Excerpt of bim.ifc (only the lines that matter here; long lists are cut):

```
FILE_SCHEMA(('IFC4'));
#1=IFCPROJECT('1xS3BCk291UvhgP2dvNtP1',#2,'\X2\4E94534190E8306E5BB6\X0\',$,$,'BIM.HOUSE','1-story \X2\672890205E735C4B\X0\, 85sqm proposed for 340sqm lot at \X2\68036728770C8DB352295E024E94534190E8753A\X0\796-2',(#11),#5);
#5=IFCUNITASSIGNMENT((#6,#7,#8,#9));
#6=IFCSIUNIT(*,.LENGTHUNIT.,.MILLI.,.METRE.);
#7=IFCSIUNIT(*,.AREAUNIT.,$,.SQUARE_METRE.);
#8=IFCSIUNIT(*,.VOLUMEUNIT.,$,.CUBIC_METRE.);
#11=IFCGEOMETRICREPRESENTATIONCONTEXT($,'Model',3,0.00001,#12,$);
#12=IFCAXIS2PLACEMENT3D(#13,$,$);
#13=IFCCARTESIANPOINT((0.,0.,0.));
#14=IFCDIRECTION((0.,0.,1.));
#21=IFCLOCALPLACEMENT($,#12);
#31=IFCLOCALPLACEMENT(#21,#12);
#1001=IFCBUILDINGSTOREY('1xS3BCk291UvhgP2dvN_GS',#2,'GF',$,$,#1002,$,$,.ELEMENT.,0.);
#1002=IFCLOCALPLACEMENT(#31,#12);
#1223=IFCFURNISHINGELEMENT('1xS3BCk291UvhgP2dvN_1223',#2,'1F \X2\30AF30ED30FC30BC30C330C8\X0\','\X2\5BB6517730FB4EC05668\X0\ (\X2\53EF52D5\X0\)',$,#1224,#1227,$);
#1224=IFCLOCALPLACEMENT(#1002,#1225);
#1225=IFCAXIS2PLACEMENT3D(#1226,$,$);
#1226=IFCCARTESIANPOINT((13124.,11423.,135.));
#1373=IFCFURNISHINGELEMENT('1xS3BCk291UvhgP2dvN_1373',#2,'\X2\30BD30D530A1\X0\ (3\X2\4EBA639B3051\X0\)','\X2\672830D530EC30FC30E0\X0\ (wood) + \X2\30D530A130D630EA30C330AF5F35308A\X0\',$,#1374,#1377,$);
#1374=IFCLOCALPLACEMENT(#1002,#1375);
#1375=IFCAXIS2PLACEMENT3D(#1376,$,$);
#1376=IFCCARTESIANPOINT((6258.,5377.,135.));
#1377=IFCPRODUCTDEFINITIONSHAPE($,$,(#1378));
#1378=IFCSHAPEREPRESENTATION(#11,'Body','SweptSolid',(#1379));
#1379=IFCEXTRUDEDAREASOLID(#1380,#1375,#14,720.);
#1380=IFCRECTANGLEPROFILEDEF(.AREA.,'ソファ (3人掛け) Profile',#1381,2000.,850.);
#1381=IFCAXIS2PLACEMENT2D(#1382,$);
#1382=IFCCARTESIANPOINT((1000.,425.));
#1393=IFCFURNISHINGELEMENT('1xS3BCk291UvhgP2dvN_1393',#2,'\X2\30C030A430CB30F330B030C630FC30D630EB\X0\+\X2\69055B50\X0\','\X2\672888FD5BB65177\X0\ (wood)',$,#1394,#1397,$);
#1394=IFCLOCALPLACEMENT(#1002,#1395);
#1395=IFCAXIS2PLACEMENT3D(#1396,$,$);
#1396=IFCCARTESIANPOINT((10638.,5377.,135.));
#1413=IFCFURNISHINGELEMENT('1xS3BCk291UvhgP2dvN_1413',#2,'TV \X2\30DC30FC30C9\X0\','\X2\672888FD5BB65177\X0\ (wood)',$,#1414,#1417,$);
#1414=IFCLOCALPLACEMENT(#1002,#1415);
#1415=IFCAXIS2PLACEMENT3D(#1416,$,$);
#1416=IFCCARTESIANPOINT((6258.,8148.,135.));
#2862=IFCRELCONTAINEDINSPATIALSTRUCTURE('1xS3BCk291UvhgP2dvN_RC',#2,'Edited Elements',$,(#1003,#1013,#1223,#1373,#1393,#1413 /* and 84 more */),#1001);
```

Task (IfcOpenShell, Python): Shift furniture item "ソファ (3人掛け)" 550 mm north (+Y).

```python
import ifcopenshell
import ifcopenshell.api.geometry
import ifcopenshell.util.placement
import ifcopenshell.util.unit

model = ifcopenshell.open("bim.ifc")
unit_scale = ifcopenshell.util.unit.calculate_unit_scale(model)

item = model.by_id(1373)
matrix = ifcopenshell.util.placement.get_local_placement(item.ObjectPlacement)
matrix[1, 3] += 0.55 / unit_scale
ifcopenshell.api.geometry.edit_object_placement(model, product=item, matrix=matrix, is_si=False)

print(ifcopenshell.util.placement.get_local_placement(item.ObjectPlacement).round(3) + 0.0)

model.write("bim_rev.ifc")
```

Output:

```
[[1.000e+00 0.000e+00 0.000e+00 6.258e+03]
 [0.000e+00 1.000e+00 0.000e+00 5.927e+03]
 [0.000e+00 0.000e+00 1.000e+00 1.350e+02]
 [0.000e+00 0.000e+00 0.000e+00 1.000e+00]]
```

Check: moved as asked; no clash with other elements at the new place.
